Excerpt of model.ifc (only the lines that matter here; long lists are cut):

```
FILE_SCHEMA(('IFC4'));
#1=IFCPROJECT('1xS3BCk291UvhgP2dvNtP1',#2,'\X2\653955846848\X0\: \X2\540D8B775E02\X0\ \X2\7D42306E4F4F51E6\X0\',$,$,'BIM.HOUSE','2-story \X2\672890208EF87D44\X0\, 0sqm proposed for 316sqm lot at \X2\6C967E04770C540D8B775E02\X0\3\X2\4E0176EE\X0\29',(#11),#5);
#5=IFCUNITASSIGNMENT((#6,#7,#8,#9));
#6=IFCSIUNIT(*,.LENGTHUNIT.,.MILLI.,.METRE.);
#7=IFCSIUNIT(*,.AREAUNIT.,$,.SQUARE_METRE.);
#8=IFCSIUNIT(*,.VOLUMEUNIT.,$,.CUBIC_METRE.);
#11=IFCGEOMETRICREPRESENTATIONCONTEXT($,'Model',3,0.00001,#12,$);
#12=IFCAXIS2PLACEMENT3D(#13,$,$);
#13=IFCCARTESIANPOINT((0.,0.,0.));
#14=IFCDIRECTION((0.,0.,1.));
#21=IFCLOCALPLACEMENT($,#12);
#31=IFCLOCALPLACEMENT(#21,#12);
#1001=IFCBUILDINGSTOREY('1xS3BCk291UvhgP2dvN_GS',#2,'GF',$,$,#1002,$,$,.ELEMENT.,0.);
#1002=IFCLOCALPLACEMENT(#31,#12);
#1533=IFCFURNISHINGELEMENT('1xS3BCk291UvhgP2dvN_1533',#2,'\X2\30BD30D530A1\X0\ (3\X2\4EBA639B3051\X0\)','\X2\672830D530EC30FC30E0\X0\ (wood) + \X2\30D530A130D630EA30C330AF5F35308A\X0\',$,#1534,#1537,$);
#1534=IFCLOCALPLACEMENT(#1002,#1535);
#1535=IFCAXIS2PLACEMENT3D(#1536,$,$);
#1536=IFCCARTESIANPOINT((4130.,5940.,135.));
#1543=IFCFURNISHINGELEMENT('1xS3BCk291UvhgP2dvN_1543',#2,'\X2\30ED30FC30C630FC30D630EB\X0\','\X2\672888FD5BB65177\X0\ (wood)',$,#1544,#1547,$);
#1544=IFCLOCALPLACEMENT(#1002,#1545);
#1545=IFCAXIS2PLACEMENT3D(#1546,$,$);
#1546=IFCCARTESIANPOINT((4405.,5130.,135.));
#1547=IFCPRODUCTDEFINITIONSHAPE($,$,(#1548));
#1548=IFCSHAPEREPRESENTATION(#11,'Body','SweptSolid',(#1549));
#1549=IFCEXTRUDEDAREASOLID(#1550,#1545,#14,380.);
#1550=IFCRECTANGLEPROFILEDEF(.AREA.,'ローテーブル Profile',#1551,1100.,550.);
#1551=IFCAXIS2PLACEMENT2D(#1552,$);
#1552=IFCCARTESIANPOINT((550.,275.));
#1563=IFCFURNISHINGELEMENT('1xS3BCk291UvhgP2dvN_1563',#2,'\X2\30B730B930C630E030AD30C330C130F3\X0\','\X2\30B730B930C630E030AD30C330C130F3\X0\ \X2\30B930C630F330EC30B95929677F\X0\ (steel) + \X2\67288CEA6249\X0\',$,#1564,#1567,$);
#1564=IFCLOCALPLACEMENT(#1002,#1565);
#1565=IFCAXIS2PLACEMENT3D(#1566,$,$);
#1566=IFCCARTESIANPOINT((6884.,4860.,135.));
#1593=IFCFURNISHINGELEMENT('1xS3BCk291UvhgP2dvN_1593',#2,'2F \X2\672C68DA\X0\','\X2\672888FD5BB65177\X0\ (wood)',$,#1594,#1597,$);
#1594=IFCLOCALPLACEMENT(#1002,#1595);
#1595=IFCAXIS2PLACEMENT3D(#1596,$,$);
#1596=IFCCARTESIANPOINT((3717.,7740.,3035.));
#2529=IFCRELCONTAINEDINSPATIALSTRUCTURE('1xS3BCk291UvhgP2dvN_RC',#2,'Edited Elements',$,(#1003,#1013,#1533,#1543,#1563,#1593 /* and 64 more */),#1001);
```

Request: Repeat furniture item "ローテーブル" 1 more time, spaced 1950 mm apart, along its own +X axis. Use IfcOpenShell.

```python
import ifcopenshell
import ifcopenshell.api.geometry
import ifcopenshell.api.root
import ifcopenshell.util.element
import ifcopenshell.util.placement
import ifcopenshell.util.unit

model = ifcopenshell.open("model.ifc")
unit_scale = ifcopenshell.util.unit.calculate_unit_scale(model)


def reuse_history(source, copy):
    """copy_class also copies each property set's owner history, people and application; keep the originals."""
    for rel in copy.IsDefinedBy:
        if rel.is_a("IfcRelDefinesByProperties") and (history := rel.RelatingPropertyDefinition.OwnerHistory):
            rel.RelatingPropertyDefinition.OwnerHistory = source.OwnerHistory
            ifcopenshell.util.element.remove_deep2(model, history)


source = model.by_guid("1xS3BCk291UvhgP2dvN_1543")
base = ifcopenshell.util.placement.get_local_placement(source.ObjectPlacement)
step = base[:3, 0] * 1.95 / unit_scale

for i in range(1, 2):
    copy = ifcopenshell.api.root.copy_class(model, product=source)
    copy.Representation = ifcopenshell.util.element.copy_deep(
        model, source.Representation, exclude=["IfcGeometricRepresentationContext", "IfcRepresentationMap"]
    )
    reuse_history(source, copy)
    matrix = base.copy()
    matrix[:3, 3] += i * step
    print("added at", matrix[:3, 3].round(3) + 0.0)
    ifcopenshell.api.geometry.edit_object_placement(model, product=copy, matrix=matrix, is_si=False)

model.write("model_v2.ifc")
```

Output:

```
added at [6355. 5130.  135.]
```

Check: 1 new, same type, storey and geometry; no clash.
